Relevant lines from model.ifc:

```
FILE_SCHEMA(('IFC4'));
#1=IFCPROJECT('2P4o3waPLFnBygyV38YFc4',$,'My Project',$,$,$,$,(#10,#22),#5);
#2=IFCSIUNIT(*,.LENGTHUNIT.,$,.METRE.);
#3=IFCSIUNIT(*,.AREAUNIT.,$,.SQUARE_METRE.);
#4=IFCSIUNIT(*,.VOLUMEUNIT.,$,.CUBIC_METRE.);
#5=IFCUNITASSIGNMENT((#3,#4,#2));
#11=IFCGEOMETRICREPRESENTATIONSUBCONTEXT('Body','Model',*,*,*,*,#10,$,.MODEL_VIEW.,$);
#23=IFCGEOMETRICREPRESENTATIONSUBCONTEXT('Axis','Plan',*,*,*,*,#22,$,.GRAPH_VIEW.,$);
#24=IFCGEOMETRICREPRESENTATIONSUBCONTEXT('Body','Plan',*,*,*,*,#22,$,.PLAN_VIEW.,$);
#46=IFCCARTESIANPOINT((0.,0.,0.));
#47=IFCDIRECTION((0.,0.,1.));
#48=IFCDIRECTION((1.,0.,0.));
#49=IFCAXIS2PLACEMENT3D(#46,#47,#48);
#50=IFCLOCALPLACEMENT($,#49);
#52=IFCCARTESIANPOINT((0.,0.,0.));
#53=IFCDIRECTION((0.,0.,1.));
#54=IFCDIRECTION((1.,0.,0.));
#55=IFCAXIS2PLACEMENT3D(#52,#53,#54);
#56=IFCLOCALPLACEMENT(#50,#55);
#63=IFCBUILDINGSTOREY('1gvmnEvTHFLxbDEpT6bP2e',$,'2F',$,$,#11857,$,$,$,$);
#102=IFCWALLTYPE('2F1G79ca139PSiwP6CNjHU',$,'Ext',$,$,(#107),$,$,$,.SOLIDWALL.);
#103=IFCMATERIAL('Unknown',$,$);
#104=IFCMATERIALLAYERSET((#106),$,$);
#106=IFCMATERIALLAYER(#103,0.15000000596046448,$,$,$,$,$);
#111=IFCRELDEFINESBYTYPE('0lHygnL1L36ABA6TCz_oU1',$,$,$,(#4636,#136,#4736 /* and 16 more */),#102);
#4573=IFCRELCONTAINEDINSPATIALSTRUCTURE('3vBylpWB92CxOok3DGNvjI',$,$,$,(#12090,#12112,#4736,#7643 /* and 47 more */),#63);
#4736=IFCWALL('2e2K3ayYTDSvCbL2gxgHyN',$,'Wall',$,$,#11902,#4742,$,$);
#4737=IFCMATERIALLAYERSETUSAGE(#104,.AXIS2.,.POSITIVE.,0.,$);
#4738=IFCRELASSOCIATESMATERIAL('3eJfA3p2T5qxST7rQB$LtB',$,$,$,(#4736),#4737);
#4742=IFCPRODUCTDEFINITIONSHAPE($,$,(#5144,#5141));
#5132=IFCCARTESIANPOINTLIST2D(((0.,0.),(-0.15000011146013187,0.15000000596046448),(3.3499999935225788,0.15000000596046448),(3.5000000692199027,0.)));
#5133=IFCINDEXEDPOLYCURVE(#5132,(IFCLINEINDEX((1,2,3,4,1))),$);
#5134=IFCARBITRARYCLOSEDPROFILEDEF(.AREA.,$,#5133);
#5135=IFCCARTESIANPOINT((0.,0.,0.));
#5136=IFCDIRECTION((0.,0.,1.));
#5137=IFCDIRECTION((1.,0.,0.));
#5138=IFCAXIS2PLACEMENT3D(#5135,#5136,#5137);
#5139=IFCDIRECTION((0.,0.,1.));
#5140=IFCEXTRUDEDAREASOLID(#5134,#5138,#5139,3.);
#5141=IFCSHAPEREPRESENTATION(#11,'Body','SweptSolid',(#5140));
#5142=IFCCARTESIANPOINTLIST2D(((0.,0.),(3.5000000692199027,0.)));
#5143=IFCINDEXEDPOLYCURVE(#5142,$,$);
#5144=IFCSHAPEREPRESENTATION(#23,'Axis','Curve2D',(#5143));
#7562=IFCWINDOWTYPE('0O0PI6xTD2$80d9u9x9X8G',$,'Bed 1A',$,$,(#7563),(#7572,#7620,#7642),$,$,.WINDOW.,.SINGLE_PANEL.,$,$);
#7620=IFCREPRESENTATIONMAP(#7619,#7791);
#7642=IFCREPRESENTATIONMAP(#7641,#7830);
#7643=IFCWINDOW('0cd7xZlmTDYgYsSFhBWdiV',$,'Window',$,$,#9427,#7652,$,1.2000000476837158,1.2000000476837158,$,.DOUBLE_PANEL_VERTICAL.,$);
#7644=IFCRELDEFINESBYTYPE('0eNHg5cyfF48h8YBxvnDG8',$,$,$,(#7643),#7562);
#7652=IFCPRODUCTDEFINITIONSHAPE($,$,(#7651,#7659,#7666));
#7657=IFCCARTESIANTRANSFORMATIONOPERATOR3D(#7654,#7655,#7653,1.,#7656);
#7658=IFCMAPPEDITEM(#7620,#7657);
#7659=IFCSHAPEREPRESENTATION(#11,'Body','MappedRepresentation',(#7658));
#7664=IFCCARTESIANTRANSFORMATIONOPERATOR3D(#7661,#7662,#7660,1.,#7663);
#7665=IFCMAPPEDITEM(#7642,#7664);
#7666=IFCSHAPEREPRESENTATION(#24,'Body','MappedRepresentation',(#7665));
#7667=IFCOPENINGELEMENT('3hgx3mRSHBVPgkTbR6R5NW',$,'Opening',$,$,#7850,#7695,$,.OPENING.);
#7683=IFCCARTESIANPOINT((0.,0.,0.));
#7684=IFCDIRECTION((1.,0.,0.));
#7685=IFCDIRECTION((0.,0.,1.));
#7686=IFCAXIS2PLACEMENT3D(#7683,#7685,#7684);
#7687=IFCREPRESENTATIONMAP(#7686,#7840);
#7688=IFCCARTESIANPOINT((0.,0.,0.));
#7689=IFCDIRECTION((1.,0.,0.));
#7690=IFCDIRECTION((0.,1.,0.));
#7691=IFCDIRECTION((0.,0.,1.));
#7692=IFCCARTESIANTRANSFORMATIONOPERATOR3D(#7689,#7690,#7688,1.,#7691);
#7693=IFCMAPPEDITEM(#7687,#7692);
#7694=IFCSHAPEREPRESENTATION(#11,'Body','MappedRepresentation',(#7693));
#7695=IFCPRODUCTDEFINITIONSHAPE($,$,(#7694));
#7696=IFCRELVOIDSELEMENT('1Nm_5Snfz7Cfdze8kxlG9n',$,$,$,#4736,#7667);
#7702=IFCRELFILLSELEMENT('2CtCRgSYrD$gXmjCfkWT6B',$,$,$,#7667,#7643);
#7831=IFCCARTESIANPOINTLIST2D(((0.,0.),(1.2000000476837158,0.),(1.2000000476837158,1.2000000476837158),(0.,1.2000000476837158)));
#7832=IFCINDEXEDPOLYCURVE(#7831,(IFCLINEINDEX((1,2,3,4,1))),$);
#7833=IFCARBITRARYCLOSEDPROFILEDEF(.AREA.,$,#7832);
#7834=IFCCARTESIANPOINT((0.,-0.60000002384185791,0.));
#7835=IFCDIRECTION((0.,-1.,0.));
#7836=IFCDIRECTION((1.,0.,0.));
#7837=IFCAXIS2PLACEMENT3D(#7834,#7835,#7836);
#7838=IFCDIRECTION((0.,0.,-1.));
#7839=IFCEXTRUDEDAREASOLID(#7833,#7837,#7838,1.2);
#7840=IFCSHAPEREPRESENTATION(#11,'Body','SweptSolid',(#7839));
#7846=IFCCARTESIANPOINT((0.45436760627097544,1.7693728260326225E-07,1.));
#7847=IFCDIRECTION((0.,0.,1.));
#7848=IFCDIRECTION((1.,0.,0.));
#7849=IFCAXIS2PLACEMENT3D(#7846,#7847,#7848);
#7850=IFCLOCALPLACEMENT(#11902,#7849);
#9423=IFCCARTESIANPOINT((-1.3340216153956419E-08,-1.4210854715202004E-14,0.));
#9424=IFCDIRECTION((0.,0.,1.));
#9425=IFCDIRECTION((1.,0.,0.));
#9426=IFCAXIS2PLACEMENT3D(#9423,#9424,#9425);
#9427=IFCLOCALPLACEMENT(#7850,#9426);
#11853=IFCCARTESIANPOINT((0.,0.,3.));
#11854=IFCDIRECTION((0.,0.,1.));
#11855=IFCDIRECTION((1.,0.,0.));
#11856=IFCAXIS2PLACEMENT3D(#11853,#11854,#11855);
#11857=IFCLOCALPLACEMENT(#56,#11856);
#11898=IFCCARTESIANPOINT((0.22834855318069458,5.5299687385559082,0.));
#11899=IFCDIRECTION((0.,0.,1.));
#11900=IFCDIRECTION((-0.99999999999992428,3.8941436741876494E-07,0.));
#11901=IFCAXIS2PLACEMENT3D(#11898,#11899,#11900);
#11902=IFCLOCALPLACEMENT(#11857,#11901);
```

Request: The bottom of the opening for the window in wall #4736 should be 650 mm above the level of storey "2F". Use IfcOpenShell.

```python
import numpy as np
import ifcopenshell
import ifcopenshell.api.geometry
import ifcopenshell.geom
import ifcopenshell.util.element
import ifcopenshell.util.placement
import ifcopenshell.util.shape
import ifcopenshell.util.unit

model = ifcopenshell.open("model.ifc")
unit_scale = ifcopenshell.util.unit.calculate_unit_scale(model)

window = model.by_guid("0cd7xZlmTDYgYsSFhBWdiV")
opening = window.FillsVoids[0].RelatingOpeningElement
storey = ifcopenshell.util.element.get_container(window, ifc_class="IfcBuildingStorey")
level = ifcopenshell.util.placement.get_local_placement(storey.ObjectPlacement)[2, 3]

# The opening's origin need not be at the sill, so measure its lowest point.
shape = ifcopenshell.geom.create_shape(ifcopenshell.geom.settings(), opening)
bottom = ifcopenshell.util.shape.get_shape_bottom_elevation(shape, shape.geometry) / unit_scale
dz = level + 0.65 / unit_scale - bottom

shift = np.array([0.0, 0.0, dz])
# The window is placed relative to its opening, so it follows when the opening moves.
matrix = ifcopenshell.util.placement.get_local_placement(opening.ObjectPlacement)
matrix[:3, 3] += shift
ifcopenshell.api.geometry.edit_object_placement(
    model, product=opening, matrix=matrix, is_si=False, should_transform_children=True
)

print(f"moved by {dz * unit_scale:+.3f} m")

model.write("model_rev.ifc")
```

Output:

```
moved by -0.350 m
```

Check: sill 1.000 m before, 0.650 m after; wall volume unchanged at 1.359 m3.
